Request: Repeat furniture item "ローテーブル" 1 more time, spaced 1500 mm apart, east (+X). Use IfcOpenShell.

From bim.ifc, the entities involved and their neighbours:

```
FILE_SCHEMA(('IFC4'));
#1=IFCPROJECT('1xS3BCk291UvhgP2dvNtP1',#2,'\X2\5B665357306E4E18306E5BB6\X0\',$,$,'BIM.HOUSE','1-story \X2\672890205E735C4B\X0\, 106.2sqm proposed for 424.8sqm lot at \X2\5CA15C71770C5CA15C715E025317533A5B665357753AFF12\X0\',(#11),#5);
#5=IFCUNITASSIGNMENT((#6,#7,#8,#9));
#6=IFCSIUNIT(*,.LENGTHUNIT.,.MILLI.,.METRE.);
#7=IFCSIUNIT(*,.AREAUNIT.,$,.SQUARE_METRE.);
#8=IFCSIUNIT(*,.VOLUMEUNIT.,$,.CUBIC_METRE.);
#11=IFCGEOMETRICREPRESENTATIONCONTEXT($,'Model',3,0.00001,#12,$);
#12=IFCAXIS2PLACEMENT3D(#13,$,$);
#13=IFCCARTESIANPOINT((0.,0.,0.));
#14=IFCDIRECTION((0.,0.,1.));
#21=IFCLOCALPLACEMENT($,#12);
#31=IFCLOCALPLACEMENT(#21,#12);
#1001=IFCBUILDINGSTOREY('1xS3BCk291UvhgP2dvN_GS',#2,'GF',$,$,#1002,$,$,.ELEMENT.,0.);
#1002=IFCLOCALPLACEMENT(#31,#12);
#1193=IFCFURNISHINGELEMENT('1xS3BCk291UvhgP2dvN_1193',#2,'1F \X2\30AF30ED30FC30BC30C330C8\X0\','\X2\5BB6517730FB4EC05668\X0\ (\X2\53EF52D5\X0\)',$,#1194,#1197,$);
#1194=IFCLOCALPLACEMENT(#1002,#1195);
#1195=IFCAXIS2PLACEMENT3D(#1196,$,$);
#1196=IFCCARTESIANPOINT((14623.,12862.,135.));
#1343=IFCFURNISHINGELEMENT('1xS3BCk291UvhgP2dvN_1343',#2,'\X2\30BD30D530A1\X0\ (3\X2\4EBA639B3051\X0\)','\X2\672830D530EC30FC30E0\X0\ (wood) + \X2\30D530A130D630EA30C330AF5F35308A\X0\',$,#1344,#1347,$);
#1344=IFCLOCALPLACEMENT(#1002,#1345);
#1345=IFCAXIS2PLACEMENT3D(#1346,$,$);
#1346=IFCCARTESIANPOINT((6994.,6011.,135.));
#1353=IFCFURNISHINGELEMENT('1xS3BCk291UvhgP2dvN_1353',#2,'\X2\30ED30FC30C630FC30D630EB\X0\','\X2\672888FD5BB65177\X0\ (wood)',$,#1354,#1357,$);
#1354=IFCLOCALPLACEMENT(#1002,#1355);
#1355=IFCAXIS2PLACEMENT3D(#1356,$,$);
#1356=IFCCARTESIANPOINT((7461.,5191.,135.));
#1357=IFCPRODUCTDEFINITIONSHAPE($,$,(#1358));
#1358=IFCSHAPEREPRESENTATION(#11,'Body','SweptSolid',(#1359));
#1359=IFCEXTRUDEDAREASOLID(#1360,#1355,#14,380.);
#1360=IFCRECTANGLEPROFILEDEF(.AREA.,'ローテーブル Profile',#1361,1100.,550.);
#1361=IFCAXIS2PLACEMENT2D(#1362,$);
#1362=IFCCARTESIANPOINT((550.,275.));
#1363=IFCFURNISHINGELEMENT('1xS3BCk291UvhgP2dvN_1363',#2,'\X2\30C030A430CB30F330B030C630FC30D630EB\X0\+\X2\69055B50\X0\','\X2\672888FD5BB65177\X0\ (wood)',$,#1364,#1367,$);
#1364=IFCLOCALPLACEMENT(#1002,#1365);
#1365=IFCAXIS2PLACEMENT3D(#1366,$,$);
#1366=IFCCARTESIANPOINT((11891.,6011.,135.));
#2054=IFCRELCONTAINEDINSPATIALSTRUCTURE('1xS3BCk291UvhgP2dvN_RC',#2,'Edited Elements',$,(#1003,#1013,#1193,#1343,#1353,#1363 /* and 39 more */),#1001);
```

```python
import numpy as np
import ifcopenshell
import ifcopenshell.api.geometry
import ifcopenshell.api.root
import ifcopenshell.util.element
import ifcopenshell.util.placement
import ifcopenshell.util.unit

model = ifcopenshell.open("bim.ifc")
unit_scale = ifcopenshell.util.unit.calculate_unit_scale(model)


def reuse_history(source, copy):
    """copy_class also copies each property set's owner history, people and application; keep the originals."""
    for rel in copy.IsDefinedBy:
        if rel.is_a("IfcRelDefinesByProperties") and (history := rel.RelatingPropertyDefinition.OwnerHistory):
            rel.RelatingPropertyDefinition.OwnerHistory = source.OwnerHistory
            ifcopenshell.util.element.remove_deep2(model, history)


source = model.by_id(1353)
base = ifcopenshell.util.placement.get_local_placement(source.ObjectPlacement)
step = np.array([1.0, 0.0, 0.0]) * 1.5 / unit_scale

for i in range(1, 2):
    copy = ifcopenshell.api.root.copy_class(model, product=source)
    copy.Representation = ifcopenshell.util.element.copy_deep(
        model, source.Representation, exclude=["IfcGeometricRepresentationContext", "IfcRepresentationMap"]
    )
    reuse_history(source, copy)
    matrix = base.copy()
    matrix[:3, 3] += i * step
    print("added at", matrix[:3, 3].round(3) + 0.0)
    ifcopenshell.api.geometry.edit_object_placement(model, product=copy, matrix=matrix, is_si=False)

model.write("bim-out.ifc")
```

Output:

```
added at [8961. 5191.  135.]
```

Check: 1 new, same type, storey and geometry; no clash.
